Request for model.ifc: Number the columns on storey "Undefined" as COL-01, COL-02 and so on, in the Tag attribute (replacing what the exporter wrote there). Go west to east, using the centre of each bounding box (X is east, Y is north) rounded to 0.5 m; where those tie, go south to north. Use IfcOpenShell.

First a look at what the model holds.

```python
import ifcopenshell
import ifcopenshell.util.element
import ifcopenshell.util.placement

model = ifcopenshell.open("model.ifc")
print(model.schema)
storey = next(s for s in model.by_type("IfcBuildingStorey") if s.Name == "Undefined")
columns = [e for e in ifcopenshell.util.element.get_decomposition(storey) if e.is_a("IfcColumn")]
for e in sorted(columns, key=lambda e: e.id()):
    origin = ifcopenshell.util.placement.get_local_placement(e.ObjectPlacement)[:3, 3]
    print(e.id(), e.Tag, e.Name, origin.round(2) + 0.0, sep=" | ")
```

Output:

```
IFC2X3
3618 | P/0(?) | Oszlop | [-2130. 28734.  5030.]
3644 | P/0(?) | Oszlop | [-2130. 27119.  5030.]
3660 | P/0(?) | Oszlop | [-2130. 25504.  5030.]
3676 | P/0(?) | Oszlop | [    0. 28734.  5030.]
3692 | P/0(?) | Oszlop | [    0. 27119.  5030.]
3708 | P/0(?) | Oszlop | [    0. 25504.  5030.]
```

```python
import ifcopenshell
import ifcopenshell.geom
import ifcopenshell.util.element
import ifcopenshell.util.shape

model = ifcopenshell.open("model.ifc")
settings = ifcopenshell.geom.settings()
settings.set("use-world-coords", True)


def centre(element):
    shape = ifcopenshell.geom.create_shape(settings, element)
    return ifcopenshell.util.shape.get_bbox_centroid(shape.geometry)


storey = next(s for s in model.by_type("IfcBuildingStorey") if s.Name == "Undefined")
columns = [e for e in ifcopenshell.util.element.get_decomposition(storey) if e.is_a("IfcColumn")]

# Insertion points can sit at a corner or the storey origin, so sort by the geometry (in metres).
centres = {e: centre(e) for e in columns}
columns.sort(key=lambda e: (round(centres[e][0] / 0.5), centres[e][1]))

for i, e in enumerate(columns, start=1):
    number = f"COL-{i:02d}"
    e.Tag = number
    print(e.id(), number)

model.write("model_edited.ifc")
```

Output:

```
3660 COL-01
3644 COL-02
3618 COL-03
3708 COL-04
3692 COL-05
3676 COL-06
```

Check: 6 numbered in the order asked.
